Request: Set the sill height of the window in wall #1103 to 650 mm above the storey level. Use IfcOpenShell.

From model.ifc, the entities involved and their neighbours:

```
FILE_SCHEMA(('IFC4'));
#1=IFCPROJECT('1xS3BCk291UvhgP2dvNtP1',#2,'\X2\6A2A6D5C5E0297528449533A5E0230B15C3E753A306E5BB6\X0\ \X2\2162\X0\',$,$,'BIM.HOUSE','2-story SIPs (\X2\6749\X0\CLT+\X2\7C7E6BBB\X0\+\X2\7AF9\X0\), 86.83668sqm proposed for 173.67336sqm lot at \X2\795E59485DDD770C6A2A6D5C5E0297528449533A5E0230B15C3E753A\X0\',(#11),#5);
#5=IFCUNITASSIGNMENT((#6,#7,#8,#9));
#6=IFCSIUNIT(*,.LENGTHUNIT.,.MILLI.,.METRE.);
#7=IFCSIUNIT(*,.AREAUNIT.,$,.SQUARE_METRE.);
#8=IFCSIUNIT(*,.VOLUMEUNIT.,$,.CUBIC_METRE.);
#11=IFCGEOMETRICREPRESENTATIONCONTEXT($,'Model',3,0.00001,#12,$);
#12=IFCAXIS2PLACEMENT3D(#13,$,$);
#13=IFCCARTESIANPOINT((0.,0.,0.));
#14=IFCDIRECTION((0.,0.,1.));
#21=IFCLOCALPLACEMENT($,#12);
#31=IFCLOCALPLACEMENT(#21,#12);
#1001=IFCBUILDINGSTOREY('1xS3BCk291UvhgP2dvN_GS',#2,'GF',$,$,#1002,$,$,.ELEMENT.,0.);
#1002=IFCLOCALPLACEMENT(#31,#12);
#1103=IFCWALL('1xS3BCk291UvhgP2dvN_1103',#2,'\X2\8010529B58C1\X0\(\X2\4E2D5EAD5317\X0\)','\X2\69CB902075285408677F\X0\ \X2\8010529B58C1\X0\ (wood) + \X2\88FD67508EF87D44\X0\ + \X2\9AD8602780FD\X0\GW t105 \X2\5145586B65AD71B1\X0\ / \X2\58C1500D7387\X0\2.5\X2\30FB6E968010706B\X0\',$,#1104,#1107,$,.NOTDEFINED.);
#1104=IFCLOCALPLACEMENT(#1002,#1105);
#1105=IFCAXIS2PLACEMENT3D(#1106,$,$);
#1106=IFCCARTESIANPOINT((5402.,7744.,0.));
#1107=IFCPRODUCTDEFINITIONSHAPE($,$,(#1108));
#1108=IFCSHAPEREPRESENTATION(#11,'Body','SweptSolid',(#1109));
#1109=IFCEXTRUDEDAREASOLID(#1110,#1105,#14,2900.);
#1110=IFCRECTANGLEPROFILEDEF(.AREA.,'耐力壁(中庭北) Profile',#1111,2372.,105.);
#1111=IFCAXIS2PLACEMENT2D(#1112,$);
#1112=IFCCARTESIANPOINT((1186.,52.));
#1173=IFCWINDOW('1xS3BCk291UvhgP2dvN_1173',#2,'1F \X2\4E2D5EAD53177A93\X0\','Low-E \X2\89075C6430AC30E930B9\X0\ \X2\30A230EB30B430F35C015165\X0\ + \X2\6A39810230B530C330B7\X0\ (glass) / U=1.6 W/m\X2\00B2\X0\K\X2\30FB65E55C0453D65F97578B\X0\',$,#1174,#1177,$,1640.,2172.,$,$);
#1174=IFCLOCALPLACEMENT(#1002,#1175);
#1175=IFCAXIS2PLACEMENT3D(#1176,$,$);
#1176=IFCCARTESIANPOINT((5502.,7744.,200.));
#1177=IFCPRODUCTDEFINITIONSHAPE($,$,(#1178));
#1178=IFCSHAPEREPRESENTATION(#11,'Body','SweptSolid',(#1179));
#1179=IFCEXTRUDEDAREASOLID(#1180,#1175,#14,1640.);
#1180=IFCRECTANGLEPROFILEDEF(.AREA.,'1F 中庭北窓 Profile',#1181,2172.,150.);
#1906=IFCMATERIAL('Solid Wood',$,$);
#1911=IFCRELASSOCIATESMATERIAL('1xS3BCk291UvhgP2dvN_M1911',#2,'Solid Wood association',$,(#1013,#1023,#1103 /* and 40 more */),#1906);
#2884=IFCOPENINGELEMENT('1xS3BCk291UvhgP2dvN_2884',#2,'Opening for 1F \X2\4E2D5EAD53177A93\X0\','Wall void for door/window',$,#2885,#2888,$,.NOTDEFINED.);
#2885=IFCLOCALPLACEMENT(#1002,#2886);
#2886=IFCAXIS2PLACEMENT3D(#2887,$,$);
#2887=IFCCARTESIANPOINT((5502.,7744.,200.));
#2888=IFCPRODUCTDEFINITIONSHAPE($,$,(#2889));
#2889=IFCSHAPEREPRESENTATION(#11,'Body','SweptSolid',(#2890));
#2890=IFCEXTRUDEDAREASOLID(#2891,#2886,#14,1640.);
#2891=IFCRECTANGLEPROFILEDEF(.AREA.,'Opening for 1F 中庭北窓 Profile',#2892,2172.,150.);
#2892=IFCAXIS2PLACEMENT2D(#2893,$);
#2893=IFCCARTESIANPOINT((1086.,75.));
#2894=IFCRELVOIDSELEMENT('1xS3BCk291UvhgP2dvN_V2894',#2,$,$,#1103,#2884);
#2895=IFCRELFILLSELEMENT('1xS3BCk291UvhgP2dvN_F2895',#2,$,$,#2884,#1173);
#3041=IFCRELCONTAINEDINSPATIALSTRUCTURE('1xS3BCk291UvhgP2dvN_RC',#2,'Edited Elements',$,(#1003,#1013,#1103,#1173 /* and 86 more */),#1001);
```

```python
import numpy as np
import ifcopenshell
import ifcopenshell.api.geometry
import ifcopenshell.geom
import ifcopenshell.util.element
import ifcopenshell.util.placement
import ifcopenshell.util.shape
import ifcopenshell.util.unit

model = ifcopenshell.open("model.ifc")
unit_scale = ifcopenshell.util.unit.calculate_unit_scale(model)

window = model.by_id(1173)
opening = window.FillsVoids[0].RelatingOpeningElement
storey = ifcopenshell.util.element.get_container(window, ifc_class="IfcBuildingStorey")
level = ifcopenshell.util.placement.get_local_placement(storey.ObjectPlacement)[2, 3]

# The opening's origin need not be at the sill, so measure its lowest point.
shape = ifcopenshell.geom.create_shape(ifcopenshell.geom.settings(), opening)
bottom = ifcopenshell.util.shape.get_shape_bottom_elevation(shape, shape.geometry) / unit_scale
dz = level + 650.0 - bottom

shift = np.array([0.0, 0.0, dz])
# The window is not placed relative to its opening, so move both.
for product in (opening, window):
    matrix = ifcopenshell.util.placement.get_local_placement(product.ObjectPlacement)
    matrix[:3, 3] += shift
    ifcopenshell.api.geometry.edit_object_placement(model, product=product, matrix=matrix, is_si=False)

print(f"moved by {dz * unit_scale:+.3f} m")

model.write("model-out.ifc")
```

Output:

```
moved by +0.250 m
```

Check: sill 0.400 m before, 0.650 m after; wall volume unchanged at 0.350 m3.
